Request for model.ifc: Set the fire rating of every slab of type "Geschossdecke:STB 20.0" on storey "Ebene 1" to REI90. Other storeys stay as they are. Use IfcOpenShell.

First a look at what the model holds.

```python
import ifcopenshell
import ifcopenshell.util.element

model = ifcopenshell.open("model.ifc")
print(model.schema)
storey = next(s for s in model.by_type("IfcBuildingStorey") if s.Name == "Ebene 1")
slabs = [e for e in ifcopenshell.util.element.get_decomposition(storey) if e.is_a("IfcSlab")]
seen = {}
for e in slabs:
    element_type = ifcopenshell.util.element.get_type(e)
    key = (element_type.Name if element_type != e and element_type else None, ifcopenshell.util.element.get_pset(e, "Pset_SlabCommon", "FireRating"))
    seen[key] = seen.get(key, 0) + 1
for (name, value), count in sorted(seen.items(), key=str):
    print(count, "x", name, "|", value)
```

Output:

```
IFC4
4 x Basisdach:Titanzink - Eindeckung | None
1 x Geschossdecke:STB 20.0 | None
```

```python
import ifcopenshell
import ifcopenshell.api.pset
import ifcopenshell.util.element

model = ifcopenshell.open("model.ifc")

storey = next(s for s in model.by_type("IfcBuildingStorey") if s.Name == "Ebene 1")
slabs = [e for e in ifcopenshell.util.element.get_decomposition(storey) if e.is_a("IfcSlab")]

count = 0
for e in slabs:
    element_type = ifcopenshell.util.element.get_type(e)
    if element_type in (None, e) or element_type.Name != "Geschossdecke:STB 20.0":
        continue
    # add_pset returns the element's existing set when there is one.
    pset = ifcopenshell.api.pset.add_pset(model, product=e, name="Pset_SlabCommon")
    ifcopenshell.api.pset.edit_pset(model, pset=pset, properties={"FireRating": "REI90"})
    count += 1

print(count, "slabs updated")

model.write("model_edited.ifc")
```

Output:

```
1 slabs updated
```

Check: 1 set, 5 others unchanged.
